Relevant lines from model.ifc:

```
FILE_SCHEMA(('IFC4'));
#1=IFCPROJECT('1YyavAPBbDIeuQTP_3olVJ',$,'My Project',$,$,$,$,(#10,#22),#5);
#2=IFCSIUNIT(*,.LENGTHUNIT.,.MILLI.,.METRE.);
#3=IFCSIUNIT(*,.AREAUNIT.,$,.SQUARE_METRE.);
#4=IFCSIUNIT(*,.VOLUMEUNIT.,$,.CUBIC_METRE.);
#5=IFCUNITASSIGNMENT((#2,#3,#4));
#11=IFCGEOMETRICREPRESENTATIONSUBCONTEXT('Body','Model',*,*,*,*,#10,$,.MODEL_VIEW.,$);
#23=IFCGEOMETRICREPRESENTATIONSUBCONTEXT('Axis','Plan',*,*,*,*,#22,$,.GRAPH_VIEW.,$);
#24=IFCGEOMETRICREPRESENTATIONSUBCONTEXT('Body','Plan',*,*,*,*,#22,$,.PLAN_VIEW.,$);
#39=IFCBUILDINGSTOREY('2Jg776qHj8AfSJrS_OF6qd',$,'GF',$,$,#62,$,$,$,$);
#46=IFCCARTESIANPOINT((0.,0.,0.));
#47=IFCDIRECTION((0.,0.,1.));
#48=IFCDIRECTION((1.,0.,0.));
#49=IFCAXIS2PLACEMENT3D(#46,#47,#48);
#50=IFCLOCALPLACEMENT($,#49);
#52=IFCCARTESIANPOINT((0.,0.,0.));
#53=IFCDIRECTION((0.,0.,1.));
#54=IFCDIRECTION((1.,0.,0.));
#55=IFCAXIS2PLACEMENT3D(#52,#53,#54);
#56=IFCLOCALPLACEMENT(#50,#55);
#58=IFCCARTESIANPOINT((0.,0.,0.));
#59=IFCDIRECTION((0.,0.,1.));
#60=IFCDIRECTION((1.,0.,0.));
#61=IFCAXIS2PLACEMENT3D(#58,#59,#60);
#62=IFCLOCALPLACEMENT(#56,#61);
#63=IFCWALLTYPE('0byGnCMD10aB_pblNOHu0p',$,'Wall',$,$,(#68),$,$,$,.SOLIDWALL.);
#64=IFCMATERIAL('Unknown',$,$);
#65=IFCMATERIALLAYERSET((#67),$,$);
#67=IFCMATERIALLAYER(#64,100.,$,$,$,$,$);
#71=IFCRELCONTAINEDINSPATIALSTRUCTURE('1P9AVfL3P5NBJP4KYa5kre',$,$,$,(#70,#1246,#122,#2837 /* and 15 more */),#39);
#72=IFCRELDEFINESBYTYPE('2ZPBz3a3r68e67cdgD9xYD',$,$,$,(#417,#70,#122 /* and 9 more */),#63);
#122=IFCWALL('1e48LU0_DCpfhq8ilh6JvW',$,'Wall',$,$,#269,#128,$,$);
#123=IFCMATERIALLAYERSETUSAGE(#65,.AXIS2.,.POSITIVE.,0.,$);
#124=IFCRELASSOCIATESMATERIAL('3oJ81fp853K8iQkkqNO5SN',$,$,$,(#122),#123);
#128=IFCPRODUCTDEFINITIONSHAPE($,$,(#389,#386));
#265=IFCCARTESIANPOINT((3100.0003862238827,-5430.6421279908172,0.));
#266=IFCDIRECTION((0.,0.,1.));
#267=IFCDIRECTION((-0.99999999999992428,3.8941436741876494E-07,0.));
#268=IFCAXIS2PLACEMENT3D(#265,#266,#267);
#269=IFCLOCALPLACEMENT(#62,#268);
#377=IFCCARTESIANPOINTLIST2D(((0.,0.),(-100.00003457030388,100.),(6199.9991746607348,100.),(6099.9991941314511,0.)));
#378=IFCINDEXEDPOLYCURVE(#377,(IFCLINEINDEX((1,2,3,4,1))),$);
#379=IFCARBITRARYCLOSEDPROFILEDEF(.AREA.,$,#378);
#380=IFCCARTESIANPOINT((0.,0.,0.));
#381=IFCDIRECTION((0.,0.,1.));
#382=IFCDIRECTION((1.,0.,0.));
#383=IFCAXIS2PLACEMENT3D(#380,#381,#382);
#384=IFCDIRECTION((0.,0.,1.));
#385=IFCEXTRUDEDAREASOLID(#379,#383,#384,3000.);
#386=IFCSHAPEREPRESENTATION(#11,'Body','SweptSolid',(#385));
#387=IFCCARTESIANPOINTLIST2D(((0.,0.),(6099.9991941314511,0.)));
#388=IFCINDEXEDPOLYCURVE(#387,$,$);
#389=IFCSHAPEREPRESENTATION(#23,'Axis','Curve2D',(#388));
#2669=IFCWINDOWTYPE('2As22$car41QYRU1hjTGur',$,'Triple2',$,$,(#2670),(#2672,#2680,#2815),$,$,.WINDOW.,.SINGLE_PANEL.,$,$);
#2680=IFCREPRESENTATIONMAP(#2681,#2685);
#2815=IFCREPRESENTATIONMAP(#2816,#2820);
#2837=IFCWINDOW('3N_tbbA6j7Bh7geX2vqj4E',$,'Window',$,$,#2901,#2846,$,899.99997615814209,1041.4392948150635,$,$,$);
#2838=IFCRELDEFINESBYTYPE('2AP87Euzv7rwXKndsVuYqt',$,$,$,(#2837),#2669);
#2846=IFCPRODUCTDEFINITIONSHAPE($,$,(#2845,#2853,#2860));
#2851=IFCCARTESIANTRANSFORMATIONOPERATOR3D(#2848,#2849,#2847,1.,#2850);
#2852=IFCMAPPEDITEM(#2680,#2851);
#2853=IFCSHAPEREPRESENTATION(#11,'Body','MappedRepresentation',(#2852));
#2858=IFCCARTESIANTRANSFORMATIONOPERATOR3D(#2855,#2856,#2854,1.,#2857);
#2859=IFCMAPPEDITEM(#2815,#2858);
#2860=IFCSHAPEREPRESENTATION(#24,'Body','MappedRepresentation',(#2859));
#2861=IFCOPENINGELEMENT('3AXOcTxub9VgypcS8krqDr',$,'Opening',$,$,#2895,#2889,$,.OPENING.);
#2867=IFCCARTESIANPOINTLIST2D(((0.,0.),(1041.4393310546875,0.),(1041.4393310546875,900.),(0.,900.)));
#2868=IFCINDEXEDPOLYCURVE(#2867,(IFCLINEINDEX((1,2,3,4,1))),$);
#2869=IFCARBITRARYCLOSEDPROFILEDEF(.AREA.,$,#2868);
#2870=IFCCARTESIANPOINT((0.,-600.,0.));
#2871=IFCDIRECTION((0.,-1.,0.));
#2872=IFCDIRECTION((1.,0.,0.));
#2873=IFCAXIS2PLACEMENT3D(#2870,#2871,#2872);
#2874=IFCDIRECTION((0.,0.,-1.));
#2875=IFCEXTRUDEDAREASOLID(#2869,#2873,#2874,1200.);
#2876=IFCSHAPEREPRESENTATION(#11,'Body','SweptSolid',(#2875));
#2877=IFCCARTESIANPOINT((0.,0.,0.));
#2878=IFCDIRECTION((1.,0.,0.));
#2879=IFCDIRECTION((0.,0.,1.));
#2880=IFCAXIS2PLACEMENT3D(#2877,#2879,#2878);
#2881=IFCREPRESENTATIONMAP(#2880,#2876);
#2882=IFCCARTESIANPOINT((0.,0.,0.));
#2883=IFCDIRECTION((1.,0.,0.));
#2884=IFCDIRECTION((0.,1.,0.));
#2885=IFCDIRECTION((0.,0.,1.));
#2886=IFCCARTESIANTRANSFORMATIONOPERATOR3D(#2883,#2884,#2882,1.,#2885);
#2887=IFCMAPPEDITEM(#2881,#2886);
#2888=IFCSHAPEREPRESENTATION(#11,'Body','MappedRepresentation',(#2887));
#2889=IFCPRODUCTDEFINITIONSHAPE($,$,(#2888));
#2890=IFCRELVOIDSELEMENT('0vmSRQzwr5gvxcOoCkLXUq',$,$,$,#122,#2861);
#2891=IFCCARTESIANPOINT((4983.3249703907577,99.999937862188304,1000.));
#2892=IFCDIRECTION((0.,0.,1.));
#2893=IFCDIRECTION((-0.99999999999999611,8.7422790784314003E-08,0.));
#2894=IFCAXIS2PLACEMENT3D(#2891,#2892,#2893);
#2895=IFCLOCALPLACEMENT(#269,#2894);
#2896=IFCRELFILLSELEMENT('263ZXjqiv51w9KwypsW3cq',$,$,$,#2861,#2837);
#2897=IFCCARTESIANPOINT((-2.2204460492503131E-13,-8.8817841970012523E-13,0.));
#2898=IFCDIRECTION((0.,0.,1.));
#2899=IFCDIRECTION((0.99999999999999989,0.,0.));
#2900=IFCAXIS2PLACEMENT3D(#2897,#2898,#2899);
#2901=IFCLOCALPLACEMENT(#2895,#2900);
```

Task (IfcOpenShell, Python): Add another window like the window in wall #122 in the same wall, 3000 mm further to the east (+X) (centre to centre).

```python
import ifcopenshell
import ifcopenshell.api.feature
import ifcopenshell.api.geometry
import ifcopenshell.api.root
import ifcopenshell.geom
import ifcopenshell.util.element
import ifcopenshell.util.placement
import ifcopenshell.util.shape
import ifcopenshell.util.unit

model = ifcopenshell.open("model.ifc")
unit_scale = ifcopenshell.util.unit.calculate_unit_scale(model)
settings = ifcopenshell.geom.settings()


def volume(element):
    """Net volume in cubic metres, openings subtracted."""
    shape = ifcopenshell.geom.create_shape(settings, element)
    return ifcopenshell.util.shape.get_volume(shape.geometry)


window = model.by_guid("3N_tbbA6j7Bh7geX2vqj4E")
opening = window.FillsVoids[0].RelatingOpeningElement
wall = opening.VoidsElements[0].RelatingBuildingElement
before = volume(wall)
shift = ifcopenshell.util.placement.get_local_placement(wall.ObjectPlacement)[:3, 0] * -3 / unit_scale

# copy_class copies the void relationship, type, container and properties, but no geometry.
new_opening = ifcopenshell.api.root.copy_class(model, product=opening)
new_opening.Representation = ifcopenshell.util.element.copy_deep(
    model, opening.Representation, exclude=["IfcGeometricRepresentationContext", "IfcRepresentationMap"]
)
new_window = ifcopenshell.api.root.copy_class(model, product=window)
new_window.Representation = ifcopenshell.util.element.copy_deep(
    model, window.Representation, exclude=["IfcGeometricRepresentationContext", "IfcRepresentationMap"]
)
ifcopenshell.api.feature.add_filling(model, opening=new_opening, element=new_window)

for old, new in ((opening, new_opening), (window, new_window)):
    matrix = ifcopenshell.util.placement.get_local_placement(old.ObjectPlacement)
    matrix[:3, 3] += shift
    ifcopenshell.api.geometry.edit_object_placement(model, product=new, matrix=matrix, is_si=False)

after = volume(wall)

print(f"wall volume {before:.3f} -> {after:.3f} m3")

model.write("model_rev.ifc")
```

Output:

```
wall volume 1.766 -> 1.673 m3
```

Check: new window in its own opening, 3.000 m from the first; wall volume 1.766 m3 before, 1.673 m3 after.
